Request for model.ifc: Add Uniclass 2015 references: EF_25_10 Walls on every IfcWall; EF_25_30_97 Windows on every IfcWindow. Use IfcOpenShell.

First a look at what the model holds.

```python
import ifcopenshell

model = ifcopenshell.open("model.ifc")
print(model.schema)
print("classifications:", [c.Name for c in model.by_type("IfcClassification")])
for ifc_class in ("IfcDoor", "IfcRoof", "IfcStair", "IfcWall", "IfcWindow"):
    print(ifc_class, len(model.by_type(ifc_class)))
```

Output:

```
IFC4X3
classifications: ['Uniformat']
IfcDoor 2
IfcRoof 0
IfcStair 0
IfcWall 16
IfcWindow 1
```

```python
import ifcopenshell
import ifcopenshell.api.classification

model = ifcopenshell.open("model.ifc")

system = ifcopenshell.api.classification.add_classification(model, classification="Uniclass 2015")

codes = {
    "IfcWall": ("EF_25_10", "Walls"),
    "IfcWindow": ("EF_25_30_97", "Windows"),
}
for ifc_class, (code, name) in codes.items():
    products = model.by_type(ifc_class)
    ifcopenshell.api.classification.add_reference(
        model, products=products, classification=system, identification=code, name=name
    )
    print(code, len(products))

model.write("model_rev.ifc")
```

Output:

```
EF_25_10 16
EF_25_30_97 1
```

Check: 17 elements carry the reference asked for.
